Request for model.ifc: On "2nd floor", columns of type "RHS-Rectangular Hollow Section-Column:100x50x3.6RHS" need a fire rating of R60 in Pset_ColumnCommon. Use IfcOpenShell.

First a look at what the model holds.

```python
import ifcopenshell
import ifcopenshell.util.element

model = ifcopenshell.open("model.ifc")
print(model.schema)
storey = next(s for s in model.by_type("IfcBuildingStorey") if s.Name == "2nd floor")
columns = [e for e in ifcopenshell.util.element.get_decomposition(storey) if e.is_a("IfcColumn")]
seen = {}
for e in columns:
    element_type = ifcopenshell.util.element.get_type(e)
    key = (element_type.Name if element_type != e and element_type else None, ifcopenshell.util.element.get_pset(e, "Pset_ColumnCommon", "FireRating"))
    seen[key] = seen.get(key, 0) + 1
for (name, value), count in sorted(seen.items(), key=str):
    print(count, "x", name, "|", value)
```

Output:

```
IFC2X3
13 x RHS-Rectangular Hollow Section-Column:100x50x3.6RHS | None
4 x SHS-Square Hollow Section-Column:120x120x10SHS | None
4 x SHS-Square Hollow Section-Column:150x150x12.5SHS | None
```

```python
import ifcopenshell
import ifcopenshell.api.pset
import ifcopenshell.util.element

model = ifcopenshell.open("model.ifc")

storey = next(s for s in model.by_type("IfcBuildingStorey") if s.Name == "2nd floor")
columns = [e for e in ifcopenshell.util.element.get_decomposition(storey) if e.is_a("IfcColumn")]

count = 0
for e in columns:
    element_type = ifcopenshell.util.element.get_type(e)
    if element_type in (None, e) or element_type.Name != "RHS-Rectangular Hollow Section-Column:100x50x3.6RHS":
        continue
    # add_pset returns the element's existing set when there is one.
    pset = ifcopenshell.api.pset.add_pset(model, product=e, name="Pset_ColumnCommon")
    ifcopenshell.api.pset.edit_pset(model, pset=pset, properties={"FireRating": "R60"})
    count += 1

print(count, "columns updated")

model.write("model_updated.ifc")
```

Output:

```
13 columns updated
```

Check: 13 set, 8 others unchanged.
